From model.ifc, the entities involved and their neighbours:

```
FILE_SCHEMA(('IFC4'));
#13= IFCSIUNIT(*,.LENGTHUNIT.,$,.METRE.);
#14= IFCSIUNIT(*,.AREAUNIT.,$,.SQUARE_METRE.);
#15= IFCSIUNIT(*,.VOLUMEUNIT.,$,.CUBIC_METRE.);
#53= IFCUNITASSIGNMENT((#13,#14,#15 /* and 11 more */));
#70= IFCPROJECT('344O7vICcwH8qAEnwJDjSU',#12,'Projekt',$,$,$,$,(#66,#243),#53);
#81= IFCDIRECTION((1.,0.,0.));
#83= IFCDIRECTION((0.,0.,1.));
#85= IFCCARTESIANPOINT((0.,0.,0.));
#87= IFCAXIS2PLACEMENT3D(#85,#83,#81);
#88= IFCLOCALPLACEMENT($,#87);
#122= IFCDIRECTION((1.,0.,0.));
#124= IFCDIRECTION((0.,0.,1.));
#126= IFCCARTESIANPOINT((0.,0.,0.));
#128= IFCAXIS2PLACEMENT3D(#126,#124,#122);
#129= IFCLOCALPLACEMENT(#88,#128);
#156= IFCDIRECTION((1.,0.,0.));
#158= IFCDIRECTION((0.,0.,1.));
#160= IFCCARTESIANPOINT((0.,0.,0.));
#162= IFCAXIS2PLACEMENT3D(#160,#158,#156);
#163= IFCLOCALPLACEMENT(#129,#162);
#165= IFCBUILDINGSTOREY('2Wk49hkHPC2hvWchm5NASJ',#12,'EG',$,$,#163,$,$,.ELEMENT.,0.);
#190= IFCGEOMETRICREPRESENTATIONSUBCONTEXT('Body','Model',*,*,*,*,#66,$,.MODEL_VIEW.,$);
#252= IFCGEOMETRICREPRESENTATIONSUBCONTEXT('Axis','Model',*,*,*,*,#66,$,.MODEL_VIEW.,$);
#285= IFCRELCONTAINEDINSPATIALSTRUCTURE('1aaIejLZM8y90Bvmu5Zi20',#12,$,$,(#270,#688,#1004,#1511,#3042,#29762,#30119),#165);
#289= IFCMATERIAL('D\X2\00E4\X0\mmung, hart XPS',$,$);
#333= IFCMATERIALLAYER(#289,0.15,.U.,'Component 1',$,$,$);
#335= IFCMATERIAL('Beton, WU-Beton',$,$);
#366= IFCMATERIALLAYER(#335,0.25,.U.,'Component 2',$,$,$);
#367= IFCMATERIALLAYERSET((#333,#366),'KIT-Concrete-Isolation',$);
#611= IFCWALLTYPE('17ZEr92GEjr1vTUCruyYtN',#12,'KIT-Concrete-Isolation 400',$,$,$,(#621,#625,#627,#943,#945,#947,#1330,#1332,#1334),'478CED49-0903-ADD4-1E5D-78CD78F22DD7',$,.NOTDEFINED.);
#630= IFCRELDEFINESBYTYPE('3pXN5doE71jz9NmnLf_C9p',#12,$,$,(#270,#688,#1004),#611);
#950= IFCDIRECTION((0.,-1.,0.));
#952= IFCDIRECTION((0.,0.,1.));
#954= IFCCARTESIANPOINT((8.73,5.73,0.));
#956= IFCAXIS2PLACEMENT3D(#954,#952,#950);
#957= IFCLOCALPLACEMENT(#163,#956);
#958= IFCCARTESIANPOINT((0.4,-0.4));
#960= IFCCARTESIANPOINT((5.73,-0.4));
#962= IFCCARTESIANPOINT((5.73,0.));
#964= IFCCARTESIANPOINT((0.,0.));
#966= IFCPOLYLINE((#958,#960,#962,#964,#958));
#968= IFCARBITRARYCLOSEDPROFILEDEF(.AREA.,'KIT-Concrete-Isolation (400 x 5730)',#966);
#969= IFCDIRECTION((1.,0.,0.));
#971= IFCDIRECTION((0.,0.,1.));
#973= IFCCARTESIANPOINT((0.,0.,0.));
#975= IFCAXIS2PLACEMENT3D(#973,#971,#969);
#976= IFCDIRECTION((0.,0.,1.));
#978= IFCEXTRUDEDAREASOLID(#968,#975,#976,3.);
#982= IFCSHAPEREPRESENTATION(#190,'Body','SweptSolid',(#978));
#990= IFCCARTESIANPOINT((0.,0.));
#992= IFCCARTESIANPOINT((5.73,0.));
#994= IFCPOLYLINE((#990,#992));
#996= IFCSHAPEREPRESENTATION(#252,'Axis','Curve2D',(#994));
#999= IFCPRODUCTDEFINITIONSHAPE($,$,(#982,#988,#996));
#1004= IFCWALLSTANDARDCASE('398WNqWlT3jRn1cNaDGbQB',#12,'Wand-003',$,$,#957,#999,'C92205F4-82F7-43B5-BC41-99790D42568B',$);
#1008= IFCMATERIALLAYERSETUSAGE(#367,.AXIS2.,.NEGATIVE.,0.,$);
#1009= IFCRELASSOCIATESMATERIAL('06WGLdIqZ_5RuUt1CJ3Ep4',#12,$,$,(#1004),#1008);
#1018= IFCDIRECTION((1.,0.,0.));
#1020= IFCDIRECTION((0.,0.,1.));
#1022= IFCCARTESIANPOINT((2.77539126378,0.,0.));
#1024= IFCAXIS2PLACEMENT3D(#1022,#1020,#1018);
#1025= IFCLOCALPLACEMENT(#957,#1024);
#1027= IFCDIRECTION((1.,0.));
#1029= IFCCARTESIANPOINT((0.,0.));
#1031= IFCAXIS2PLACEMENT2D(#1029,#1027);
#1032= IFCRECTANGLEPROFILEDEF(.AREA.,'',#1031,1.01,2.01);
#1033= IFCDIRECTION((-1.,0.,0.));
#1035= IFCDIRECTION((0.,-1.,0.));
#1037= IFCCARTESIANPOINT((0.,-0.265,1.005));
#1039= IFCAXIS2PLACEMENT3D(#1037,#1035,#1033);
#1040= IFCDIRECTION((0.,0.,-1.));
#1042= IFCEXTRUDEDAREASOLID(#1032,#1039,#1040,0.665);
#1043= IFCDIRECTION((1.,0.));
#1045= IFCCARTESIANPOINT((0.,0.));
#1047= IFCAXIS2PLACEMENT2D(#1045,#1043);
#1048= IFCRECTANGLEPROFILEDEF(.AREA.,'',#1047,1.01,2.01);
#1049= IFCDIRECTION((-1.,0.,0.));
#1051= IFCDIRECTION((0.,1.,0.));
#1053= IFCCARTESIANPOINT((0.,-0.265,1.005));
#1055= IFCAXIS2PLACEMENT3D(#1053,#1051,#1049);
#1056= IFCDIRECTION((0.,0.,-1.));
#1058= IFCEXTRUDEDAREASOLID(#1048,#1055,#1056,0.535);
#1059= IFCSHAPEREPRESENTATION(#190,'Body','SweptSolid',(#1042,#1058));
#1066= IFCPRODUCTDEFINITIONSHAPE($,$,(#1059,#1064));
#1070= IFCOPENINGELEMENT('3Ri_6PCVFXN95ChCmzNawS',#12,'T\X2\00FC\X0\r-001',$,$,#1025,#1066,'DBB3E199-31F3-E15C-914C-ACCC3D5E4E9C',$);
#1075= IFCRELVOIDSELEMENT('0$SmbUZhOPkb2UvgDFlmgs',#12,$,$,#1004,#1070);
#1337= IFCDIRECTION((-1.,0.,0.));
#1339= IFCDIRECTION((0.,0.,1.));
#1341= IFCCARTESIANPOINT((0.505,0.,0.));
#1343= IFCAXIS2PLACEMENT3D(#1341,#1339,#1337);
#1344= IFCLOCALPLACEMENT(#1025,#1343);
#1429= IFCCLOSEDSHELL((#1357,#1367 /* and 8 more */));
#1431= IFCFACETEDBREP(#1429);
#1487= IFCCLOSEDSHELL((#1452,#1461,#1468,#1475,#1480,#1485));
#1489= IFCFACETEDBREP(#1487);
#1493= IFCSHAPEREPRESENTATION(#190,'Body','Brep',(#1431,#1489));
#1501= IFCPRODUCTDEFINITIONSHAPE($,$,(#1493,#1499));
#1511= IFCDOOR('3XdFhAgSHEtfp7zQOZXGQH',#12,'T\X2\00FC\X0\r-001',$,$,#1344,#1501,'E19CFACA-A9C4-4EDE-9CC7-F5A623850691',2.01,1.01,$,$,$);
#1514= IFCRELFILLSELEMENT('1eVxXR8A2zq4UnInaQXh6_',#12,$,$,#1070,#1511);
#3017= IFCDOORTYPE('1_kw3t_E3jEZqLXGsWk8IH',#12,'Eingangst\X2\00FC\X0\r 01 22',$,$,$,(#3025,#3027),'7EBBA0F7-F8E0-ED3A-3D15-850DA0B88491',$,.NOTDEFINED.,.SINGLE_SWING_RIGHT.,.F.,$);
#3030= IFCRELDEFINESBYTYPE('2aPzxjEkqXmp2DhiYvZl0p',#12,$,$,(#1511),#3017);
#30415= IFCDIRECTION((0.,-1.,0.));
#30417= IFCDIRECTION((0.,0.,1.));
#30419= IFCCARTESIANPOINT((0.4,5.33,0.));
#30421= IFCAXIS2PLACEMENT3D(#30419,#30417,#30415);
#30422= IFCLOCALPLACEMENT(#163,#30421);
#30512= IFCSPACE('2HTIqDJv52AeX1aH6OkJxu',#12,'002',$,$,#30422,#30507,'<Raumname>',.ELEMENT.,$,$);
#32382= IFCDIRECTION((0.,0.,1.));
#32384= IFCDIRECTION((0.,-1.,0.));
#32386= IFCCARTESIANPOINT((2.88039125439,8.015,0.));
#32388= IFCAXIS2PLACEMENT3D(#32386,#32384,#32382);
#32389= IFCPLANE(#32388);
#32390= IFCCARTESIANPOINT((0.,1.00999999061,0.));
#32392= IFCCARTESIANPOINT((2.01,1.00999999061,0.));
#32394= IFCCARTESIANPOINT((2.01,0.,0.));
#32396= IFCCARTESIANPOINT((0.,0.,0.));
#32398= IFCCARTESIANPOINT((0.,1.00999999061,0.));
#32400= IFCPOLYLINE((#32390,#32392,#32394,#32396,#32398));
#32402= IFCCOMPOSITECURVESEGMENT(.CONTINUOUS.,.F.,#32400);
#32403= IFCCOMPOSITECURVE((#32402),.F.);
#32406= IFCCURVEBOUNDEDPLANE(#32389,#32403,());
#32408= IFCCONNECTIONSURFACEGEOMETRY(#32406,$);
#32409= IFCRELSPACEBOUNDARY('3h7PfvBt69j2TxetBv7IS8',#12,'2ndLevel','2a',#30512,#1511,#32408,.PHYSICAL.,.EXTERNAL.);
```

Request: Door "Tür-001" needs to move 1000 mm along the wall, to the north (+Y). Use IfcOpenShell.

```python
import numpy as np
import ifcopenshell
import ifcopenshell.api.geometry
import ifcopenshell.util.placement

model = ifcopenshell.open("model.ifc")

door = model.by_guid("3XdFhAgSHEtfp7zQOZXGQH")
opening = door.FillsVoids[0].RelatingOpeningElement
wall = opening.VoidsElements[0].RelatingBuildingElement

wall_matrix = ifcopenshell.util.placement.get_local_placement(wall.ObjectPlacement)
shift = wall_matrix[:3, 0] * -1.0
before = ifcopenshell.util.placement.get_local_placement(door.ObjectPlacement)[:3, 3].copy()

# The door is placed relative to its opening, so it follows when the opening moves.
matrix = ifcopenshell.util.placement.get_local_placement(opening.ObjectPlacement)
matrix[:3, 3] += shift
ifcopenshell.api.geometry.edit_object_placement(
    model, product=opening, matrix=matrix, is_si=False, should_transform_children=True
)

# Space boundary surfaces are stored in each space's coordinates; move them too.
for rel in door.ProvidesBoundaries:
    if not rel.ConnectionGeometry:
        continue
    surface = rel.ConnectionGeometry.SurfaceOnRelatingElement.BasisSurface
    space_matrix = ifcopenshell.util.placement.get_local_placement(rel.RelatingSpace.ObjectPlacement)
    point = np.array(surface.Position.Location.Coordinates) + space_matrix[:3, :3].T @ shift
    surface.Position = model.createIfcAxis2Placement3D(
        model.createIfcCartesianPoint(point.tolist()), surface.Position.Axis, surface.Position.RefDirection
    )

after = ifcopenshell.util.placement.get_local_placement(door.ObjectPlacement)[:3, 3]
print("door moved by", (after - before).round(3) + 0.0)

model.write("model_updated.ifc")
```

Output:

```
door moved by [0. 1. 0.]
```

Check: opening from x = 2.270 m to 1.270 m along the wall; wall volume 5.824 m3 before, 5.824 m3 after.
